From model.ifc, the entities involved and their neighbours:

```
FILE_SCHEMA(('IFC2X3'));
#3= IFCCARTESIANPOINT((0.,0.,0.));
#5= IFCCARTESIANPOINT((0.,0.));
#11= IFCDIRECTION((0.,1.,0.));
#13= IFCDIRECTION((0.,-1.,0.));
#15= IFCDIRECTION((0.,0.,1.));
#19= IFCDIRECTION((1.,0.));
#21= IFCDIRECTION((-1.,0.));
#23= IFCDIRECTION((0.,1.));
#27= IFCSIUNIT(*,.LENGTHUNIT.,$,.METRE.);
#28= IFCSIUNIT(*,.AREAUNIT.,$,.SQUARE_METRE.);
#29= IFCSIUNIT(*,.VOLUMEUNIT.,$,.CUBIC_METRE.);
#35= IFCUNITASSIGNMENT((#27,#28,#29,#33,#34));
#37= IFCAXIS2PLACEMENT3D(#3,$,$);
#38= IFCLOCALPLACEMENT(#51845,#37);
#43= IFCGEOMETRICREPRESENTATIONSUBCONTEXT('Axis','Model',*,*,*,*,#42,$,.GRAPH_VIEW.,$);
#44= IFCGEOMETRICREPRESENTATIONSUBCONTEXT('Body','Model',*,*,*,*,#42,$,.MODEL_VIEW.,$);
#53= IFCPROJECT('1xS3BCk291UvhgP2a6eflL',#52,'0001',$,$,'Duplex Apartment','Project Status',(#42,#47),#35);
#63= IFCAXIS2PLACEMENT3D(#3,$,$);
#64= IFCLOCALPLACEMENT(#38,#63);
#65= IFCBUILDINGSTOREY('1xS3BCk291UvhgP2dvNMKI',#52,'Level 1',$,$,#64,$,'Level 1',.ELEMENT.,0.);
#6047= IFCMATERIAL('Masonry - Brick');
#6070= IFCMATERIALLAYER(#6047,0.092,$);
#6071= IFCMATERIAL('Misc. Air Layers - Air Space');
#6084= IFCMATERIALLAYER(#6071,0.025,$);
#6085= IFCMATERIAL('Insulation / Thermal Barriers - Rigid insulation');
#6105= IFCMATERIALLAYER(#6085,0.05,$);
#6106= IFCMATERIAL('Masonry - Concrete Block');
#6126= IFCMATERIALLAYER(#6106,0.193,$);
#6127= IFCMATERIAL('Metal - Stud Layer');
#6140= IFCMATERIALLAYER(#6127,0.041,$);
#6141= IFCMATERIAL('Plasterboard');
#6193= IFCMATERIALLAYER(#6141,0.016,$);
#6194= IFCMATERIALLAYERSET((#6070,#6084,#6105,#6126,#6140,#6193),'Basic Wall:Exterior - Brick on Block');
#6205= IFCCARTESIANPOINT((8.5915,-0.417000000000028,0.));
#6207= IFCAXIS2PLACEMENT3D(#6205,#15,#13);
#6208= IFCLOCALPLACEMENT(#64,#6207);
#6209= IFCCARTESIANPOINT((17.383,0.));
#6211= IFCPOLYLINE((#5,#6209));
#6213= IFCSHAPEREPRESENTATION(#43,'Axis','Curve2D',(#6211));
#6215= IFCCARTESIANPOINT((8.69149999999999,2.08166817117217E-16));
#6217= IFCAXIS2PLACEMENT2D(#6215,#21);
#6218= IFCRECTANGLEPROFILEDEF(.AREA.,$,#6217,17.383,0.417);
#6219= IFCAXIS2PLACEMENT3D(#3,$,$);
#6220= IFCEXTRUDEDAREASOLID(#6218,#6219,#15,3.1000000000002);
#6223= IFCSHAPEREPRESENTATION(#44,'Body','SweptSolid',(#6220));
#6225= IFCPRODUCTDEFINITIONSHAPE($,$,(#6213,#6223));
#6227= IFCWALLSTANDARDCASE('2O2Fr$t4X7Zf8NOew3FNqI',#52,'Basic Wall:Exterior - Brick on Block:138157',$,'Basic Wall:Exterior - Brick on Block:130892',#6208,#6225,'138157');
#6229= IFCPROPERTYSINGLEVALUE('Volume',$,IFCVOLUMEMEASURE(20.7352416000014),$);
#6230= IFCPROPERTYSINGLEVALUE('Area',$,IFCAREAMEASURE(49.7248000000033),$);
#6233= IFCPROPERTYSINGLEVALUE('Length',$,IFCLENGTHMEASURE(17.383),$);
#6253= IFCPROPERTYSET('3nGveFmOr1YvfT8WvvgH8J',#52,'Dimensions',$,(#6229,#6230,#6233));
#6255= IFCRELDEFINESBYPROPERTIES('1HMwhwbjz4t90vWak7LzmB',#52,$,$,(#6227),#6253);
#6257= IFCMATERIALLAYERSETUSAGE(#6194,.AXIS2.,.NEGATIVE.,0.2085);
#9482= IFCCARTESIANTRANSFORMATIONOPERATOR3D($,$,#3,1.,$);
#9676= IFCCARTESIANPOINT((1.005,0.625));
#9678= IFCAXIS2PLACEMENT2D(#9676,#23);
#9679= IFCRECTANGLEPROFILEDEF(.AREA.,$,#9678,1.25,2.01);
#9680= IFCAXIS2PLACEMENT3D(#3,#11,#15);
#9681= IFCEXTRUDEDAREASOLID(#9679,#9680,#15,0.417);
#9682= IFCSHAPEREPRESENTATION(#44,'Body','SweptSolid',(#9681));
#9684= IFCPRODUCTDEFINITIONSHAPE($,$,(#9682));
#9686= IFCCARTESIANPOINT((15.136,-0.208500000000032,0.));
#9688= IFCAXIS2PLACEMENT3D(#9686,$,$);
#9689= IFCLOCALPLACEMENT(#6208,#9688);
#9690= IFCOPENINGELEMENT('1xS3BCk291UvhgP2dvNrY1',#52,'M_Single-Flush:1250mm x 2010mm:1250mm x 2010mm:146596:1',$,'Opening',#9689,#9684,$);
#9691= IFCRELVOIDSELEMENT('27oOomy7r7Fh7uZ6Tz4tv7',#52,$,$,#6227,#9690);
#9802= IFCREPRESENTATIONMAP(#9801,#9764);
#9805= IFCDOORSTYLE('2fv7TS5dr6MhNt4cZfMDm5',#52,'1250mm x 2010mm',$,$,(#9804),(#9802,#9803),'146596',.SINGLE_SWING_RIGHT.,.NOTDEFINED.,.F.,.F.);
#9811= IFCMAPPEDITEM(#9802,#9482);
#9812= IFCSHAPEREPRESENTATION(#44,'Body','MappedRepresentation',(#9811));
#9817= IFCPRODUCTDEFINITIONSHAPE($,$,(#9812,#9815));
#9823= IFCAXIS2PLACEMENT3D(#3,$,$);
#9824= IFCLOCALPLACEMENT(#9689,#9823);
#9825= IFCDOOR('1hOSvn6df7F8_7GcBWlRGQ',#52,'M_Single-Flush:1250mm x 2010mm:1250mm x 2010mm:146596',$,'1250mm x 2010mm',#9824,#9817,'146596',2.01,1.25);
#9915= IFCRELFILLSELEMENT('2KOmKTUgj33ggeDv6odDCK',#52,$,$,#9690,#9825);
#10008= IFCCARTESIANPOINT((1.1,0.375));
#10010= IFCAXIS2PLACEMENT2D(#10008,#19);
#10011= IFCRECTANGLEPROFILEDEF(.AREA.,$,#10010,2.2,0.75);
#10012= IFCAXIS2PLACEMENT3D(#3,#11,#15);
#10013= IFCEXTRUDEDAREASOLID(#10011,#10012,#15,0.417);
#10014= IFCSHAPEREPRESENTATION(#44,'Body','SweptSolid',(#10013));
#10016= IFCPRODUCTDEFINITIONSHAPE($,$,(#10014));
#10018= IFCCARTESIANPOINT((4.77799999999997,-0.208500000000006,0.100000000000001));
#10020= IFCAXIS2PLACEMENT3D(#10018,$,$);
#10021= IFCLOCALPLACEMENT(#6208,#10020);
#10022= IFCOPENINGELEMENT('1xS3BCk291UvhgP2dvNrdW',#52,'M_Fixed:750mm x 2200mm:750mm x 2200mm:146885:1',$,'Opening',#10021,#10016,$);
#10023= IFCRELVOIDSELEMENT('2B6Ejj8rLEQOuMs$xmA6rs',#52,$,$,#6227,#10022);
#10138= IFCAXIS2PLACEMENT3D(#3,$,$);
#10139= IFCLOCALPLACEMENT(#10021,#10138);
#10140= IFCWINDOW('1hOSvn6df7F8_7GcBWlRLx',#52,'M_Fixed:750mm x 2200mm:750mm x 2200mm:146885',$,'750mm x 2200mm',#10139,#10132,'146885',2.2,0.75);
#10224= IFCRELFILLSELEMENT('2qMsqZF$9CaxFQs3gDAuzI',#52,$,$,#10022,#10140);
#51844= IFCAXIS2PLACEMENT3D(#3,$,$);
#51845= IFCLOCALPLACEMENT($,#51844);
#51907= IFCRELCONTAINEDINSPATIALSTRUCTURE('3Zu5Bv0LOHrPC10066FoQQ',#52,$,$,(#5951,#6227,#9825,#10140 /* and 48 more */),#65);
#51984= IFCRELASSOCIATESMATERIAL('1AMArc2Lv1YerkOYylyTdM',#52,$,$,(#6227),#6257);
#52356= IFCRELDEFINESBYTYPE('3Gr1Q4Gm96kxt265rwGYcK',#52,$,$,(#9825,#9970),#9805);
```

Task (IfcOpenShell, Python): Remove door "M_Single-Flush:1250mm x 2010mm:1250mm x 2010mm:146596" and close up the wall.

```python
import ifcopenshell
import ifcopenshell.api.feature
import ifcopenshell.api.pset
import ifcopenshell.api.root
import ifcopenshell.geom
import ifcopenshell.util.element
import ifcopenshell.util.shape
import ifcopenshell.util.unit

model = ifcopenshell.open("model.ifc")
area_scale = ifcopenshell.util.unit.calculate_unit_scale(model, "AREAUNIT")
volume_scale = ifcopenshell.util.unit.calculate_unit_scale(model, "VOLUMEUNIT")
settings = ifcopenshell.geom.settings()


def volume(element):
    """Net volume in cubic metres, openings subtracted."""
    shape = ifcopenshell.geom.create_shape(settings, element)
    return ifcopenshell.util.shape.get_volume(shape.geometry)


door = model.by_id(9825)
opening = door.FillsVoids[0].RelatingOpeningElement
wall = opening.VoidsElements[0].RelatingBuildingElement
before = volume(wall)

ifcopenshell.api.root.remove_product(model, product=door)
ifcopenshell.api.feature.remove_feature(model, feature=opening)

after = volume(wall)
thickness = 0.417  # wall thickness in metres

# Update the wall's stored quantities.
pset = model.by_id(ifcopenshell.util.element.get_pset(wall, "Dimensions", should_inherit=False)["id"])
ifcopenshell.api.pset.edit_pset(model, pset=pset, properties={
    "Volume": model.create_entity("IfcVolumeMeasure", after / volume_scale),
    "Area": model.create_entity("IfcAreaMeasure", after / thickness / area_scale),
})

print(f"wall volume {before:.3f} -> {after:.3f} m3")

model.write("model-out.ifc")
```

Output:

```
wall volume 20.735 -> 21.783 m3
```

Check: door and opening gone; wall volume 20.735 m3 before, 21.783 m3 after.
